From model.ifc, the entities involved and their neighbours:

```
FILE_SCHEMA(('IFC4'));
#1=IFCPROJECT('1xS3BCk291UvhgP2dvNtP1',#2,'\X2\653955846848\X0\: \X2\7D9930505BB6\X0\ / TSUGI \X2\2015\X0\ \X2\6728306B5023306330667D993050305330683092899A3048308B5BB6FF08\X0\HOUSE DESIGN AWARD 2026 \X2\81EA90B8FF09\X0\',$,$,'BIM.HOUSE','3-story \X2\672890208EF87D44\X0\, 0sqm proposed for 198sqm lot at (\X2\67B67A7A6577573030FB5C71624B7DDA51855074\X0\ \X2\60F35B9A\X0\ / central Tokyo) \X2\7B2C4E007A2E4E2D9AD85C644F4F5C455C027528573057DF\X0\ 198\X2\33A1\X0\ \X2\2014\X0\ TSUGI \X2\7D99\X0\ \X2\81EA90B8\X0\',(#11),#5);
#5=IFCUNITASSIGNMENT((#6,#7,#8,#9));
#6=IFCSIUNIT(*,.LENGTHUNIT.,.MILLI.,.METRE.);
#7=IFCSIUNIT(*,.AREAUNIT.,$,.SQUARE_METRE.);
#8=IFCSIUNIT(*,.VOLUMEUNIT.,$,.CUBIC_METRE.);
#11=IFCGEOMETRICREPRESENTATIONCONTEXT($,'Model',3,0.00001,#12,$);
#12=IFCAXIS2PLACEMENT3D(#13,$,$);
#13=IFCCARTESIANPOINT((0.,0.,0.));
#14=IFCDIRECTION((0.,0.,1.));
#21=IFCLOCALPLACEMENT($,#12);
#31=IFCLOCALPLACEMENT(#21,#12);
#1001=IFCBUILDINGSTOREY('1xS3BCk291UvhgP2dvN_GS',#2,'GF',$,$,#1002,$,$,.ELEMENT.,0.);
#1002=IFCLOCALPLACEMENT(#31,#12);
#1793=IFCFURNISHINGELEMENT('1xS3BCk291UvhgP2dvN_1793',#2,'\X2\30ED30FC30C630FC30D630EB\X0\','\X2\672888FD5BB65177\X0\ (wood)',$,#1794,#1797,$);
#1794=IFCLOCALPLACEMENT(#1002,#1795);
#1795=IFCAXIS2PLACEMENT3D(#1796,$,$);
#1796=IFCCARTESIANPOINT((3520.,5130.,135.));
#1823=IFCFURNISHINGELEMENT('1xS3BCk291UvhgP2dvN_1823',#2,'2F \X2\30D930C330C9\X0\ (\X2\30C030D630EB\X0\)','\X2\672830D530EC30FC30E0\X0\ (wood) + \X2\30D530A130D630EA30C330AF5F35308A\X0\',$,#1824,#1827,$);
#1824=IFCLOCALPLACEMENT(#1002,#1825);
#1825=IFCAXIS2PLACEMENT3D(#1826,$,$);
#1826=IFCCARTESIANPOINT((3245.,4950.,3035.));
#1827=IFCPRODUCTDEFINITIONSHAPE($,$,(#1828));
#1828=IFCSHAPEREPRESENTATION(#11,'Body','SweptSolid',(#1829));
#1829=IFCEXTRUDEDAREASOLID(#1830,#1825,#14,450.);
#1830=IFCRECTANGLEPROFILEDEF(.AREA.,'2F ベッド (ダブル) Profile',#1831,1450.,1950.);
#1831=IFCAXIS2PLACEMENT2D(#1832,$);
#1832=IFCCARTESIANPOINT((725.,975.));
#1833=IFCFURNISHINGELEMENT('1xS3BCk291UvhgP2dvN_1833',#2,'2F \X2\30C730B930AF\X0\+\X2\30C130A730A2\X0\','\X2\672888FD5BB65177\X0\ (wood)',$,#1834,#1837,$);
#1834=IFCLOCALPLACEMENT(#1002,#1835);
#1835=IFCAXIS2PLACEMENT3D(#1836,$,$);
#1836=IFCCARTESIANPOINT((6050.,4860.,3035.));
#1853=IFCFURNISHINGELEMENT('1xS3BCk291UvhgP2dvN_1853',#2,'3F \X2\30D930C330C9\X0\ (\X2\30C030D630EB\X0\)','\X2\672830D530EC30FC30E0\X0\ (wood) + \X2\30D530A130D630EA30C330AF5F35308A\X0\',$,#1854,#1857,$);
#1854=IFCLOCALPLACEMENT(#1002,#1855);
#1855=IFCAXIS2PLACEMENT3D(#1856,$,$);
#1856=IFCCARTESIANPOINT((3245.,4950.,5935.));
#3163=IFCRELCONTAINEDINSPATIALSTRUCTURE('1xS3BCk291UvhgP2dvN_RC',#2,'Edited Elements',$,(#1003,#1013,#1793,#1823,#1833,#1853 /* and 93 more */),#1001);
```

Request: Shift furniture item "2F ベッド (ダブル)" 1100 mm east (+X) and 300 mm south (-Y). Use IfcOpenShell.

```python
import ifcopenshell
import ifcopenshell.api.geometry
import ifcopenshell.util.placement
import ifcopenshell.util.unit

model = ifcopenshell.open("model.ifc")
unit_scale = ifcopenshell.util.unit.calculate_unit_scale(model)

item = model.by_guid("1xS3BCk291UvhgP2dvN_1823")
matrix = ifcopenshell.util.placement.get_local_placement(item.ObjectPlacement)
matrix[0, 3] += 1.1 / unit_scale
matrix[1, 3] -= 0.3 / unit_scale
ifcopenshell.api.geometry.edit_object_placement(model, product=item, matrix=matrix, is_si=False)

print(ifcopenshell.util.placement.get_local_placement(item.ObjectPlacement).round(3) + 0.0)

model.write("model_rev.ifc")
```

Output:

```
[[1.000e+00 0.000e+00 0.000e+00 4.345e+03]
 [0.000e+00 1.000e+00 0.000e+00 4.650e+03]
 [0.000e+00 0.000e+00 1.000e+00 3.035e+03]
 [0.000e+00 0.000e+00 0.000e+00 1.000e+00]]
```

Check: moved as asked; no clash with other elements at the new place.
